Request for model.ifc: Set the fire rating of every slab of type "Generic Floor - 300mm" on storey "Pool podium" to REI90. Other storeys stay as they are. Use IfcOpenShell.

First a look at what the model holds.

```python
import ifcopenshell
import ifcopenshell.util.element

model = ifcopenshell.open("model.ifc")
print(model.schema)
storey = next(s for s in model.by_type("IfcBuildingStorey") if s.Name == "Pool podium")
slabs = [e for e in ifcopenshell.util.element.get_decomposition(storey) if e.is_a("IfcSlab")]
seen = {}
for e in slabs:
    element_type = ifcopenshell.util.element.get_type(e)
    key = (element_type.Name if element_type != e and element_type else None, ifcopenshell.util.element.get_pset(e, "Pset_SlabCommon", "FireRating"))
    seen[key] = seen.get(key, 0) + 1
for (name, value), count in sorted(seen.items(), key=str):
    print(count, "x", name, "|", value)
```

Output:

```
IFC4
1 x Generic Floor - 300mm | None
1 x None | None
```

```python
import ifcopenshell
import ifcopenshell.api.pset
import ifcopenshell.util.element

model = ifcopenshell.open("model.ifc")

storey = next(s for s in model.by_type("IfcBuildingStorey") if s.Name == "Pool podium")
slabs = [e for e in ifcopenshell.util.element.get_decomposition(storey) if e.is_a("IfcSlab")]

count = 0
for e in slabs:
    element_type = ifcopenshell.util.element.get_type(e)
    if element_type in (None, e) or element_type.Name != "Generic Floor - 300mm":
        continue
    # add_pset returns the element's existing set when there is one.
    pset = ifcopenshell.api.pset.add_pset(model, product=e, name="Pset_SlabCommon")
    ifcopenshell.api.pset.edit_pset(model, pset=pset, properties={"FireRating": "REI90"})
    count += 1

print(count, "slabs updated")

model.write("model_updated.ifc")
```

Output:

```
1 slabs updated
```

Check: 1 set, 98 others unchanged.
